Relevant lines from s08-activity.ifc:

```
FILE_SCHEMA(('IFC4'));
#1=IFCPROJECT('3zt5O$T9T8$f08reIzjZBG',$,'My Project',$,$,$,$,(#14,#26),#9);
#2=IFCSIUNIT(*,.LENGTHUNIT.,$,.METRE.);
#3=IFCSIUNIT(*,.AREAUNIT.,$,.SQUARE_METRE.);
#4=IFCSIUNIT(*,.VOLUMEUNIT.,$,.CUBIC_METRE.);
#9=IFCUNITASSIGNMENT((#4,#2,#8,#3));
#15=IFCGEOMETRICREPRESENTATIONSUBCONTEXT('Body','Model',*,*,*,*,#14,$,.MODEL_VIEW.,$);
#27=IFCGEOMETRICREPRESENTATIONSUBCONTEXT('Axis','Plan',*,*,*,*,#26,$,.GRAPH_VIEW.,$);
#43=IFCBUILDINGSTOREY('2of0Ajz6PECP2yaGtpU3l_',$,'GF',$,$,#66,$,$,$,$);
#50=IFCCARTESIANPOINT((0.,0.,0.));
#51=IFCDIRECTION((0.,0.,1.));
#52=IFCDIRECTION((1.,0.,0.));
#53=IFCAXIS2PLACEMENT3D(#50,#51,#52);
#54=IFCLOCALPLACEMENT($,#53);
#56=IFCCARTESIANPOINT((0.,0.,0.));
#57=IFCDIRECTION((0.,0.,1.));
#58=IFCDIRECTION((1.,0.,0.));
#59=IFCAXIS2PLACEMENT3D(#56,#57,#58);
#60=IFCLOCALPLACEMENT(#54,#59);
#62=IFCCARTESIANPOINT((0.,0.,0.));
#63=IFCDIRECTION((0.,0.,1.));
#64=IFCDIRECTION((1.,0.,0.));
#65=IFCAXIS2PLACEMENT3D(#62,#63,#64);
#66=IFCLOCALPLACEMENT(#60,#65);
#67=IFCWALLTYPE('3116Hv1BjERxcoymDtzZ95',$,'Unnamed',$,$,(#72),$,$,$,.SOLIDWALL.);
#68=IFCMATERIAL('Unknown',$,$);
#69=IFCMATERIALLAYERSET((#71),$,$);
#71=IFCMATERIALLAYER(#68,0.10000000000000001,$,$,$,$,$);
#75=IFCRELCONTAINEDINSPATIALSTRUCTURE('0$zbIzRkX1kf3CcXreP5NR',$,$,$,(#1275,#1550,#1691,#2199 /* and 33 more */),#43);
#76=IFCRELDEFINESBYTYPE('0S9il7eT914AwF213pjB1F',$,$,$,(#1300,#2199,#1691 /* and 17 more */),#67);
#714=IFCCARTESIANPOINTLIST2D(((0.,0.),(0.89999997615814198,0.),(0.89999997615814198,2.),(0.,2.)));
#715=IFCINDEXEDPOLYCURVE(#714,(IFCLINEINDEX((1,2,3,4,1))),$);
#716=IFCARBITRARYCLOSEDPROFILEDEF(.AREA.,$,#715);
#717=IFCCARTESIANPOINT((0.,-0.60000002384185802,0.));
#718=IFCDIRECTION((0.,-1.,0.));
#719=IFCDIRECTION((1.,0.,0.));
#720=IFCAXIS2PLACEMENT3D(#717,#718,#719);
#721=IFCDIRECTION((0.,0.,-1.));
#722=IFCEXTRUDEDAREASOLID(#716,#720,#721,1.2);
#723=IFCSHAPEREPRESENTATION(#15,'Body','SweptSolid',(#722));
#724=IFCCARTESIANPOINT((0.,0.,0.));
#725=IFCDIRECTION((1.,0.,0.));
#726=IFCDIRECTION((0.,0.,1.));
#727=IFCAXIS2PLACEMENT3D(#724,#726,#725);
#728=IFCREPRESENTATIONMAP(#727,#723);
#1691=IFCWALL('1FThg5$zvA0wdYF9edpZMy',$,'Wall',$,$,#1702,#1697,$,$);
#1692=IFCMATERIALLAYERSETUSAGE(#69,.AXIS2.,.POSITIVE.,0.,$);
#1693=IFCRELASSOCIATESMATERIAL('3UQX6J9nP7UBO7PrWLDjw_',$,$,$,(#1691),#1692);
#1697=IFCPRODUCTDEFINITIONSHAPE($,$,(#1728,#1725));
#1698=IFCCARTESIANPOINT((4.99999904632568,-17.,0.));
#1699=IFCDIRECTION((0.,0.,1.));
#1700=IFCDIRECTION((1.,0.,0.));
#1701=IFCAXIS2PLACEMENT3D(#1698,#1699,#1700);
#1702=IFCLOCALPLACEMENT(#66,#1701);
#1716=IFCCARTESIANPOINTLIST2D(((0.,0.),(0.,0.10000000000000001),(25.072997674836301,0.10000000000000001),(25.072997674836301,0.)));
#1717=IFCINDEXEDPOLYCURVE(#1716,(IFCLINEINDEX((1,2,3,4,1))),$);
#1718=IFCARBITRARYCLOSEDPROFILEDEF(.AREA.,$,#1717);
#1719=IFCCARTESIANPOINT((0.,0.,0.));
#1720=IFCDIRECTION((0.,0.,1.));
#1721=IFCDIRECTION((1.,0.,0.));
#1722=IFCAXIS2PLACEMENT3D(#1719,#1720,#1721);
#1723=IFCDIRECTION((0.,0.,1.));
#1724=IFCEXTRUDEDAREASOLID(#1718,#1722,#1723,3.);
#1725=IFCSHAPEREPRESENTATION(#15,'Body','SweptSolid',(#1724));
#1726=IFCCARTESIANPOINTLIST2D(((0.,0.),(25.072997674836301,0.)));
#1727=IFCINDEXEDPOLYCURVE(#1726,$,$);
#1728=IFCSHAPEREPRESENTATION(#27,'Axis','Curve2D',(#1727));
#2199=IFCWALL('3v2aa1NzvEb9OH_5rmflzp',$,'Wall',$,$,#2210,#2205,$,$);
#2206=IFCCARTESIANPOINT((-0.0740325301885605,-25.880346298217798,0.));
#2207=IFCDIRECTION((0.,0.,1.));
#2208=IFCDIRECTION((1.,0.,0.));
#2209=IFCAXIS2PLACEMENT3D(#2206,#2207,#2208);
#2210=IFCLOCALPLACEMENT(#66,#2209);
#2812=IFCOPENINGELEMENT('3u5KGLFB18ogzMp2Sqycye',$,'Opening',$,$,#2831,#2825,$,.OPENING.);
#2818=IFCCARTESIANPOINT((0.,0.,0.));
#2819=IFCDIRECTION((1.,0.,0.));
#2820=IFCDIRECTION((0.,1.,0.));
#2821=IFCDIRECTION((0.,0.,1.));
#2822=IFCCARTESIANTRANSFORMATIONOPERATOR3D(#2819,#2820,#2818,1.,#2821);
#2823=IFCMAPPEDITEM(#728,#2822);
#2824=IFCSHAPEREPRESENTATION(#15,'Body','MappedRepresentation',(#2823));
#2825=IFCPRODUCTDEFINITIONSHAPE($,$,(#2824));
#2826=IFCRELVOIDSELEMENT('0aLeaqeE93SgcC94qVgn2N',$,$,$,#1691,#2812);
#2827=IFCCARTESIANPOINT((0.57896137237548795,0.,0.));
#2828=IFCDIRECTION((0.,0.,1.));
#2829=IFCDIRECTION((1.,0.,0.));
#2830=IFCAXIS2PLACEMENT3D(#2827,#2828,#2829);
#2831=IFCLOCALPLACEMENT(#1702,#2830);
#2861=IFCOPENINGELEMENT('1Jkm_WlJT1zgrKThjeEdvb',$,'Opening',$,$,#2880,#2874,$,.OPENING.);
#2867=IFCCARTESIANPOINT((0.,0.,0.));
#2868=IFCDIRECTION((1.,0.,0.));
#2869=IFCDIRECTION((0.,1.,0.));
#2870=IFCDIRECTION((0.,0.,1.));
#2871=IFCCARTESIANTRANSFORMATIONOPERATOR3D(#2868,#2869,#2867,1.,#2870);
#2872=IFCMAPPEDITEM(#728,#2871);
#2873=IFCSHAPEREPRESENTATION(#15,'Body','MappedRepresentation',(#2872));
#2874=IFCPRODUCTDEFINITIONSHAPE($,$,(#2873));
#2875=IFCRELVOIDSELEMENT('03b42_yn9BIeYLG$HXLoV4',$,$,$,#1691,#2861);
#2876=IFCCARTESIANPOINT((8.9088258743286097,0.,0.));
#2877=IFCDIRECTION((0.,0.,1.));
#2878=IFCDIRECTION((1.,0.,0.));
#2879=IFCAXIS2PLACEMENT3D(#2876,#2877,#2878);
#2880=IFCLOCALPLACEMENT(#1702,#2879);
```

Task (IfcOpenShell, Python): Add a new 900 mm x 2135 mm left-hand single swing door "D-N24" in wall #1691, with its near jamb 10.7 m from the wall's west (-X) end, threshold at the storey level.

```python
import numpy as np
import ifcopenshell
import ifcopenshell.api.feature
import ifcopenshell.api.geometry
import ifcopenshell.api.root
import ifcopenshell.api.spatial
import ifcopenshell.geom
import ifcopenshell.util.element
import ifcopenshell.util.placement
import ifcopenshell.util.representation
import ifcopenshell.util.shape
import ifcopenshell.util.unit

model = ifcopenshell.open("s08-activity.ifc")
unit_scale = ifcopenshell.util.unit.calculate_unit_scale(model)
settings = ifcopenshell.geom.settings()


def volume(element):
    """Net volume in cubic metres, openings subtracted."""
    shape = ifcopenshell.geom.create_shape(settings, element)
    return ifcopenshell.util.shape.get_volume(shape.geometry)


wall = model.by_guid("1FThg5$zvA0wdYF9edpZMy")
storey = ifcopenshell.util.element.get_container(wall, ifc_class="IfcBuildingStorey")
context = ifcopenshell.util.representation.get_context(model, "Model", "Body", "MODEL_VIEW")
before = volume(wall)

width, height, from_end, sill = 0.9, 2.135, 10.7, 0.0  # metres

# The wall runs along its own X axis, and the end named is its -X end.
wall_shape = ifcopenshell.geom.create_shape(settings, wall)
x, y, z = ifcopenshell.util.shape.get_vertices(wall_shape.geometry).T
start = x.min() + from_end
face, thickness = float(y.min()), float(y.max() - y.min())
wall_matrix = ifcopenshell.util.placement.get_local_placement(wall.ObjectPlacement)
level = ifcopenshell.util.placement.get_local_placement(storey.ObjectPlacement)[2, 3]


def in_wall(x, y):
    """Placement at x, y metres in the wall's axes, at sill height."""
    matrix = wall_matrix.copy()
    matrix[:, 3] = wall_matrix @ np.array([x / unit_scale, y / unit_scale, 0.0, 1.0])
    matrix[2, 3] = level + sill / unit_scale
    return matrix


# Opening: a box that overshoots both wall faces by 50 mm.
opening = ifcopenshell.api.root.create_entity(model, ifc_class="IfcOpeningElement", predefined_type="OPENING")
box = ifcopenshell.api.geometry.add_wall_representation(
    model, context=context, length=width, height=height, thickness=thickness + 0.1
)
ifcopenshell.api.geometry.assign_representation(model, product=opening, representation=box)
ifcopenshell.api.geometry.edit_object_placement(model, product=opening, matrix=in_wall(start, face - 0.05), is_si=False)
ifcopenshell.api.feature.add_feature(model, feature=opening, element=wall)

door = ifcopenshell.api.root.create_entity(model, ifc_class="IfcDoor", name="D-N24", predefined_type="DOOR")
door.OverallWidth, door.OverallHeight = width / unit_scale, height / unit_scale
door.OperationType = "SINGLE_SWING_LEFT"
body = ifcopenshell.api.geometry.add_door_representation(
    model,
    context=context,
    overall_width=door.OverallWidth,
    overall_height=door.OverallHeight,
    operation_type="SINGLE_SWING_LEFT",
    lining_properties={"LiningDepth": thickness / unit_scale, "ThresholdDepth": thickness / unit_scale},
)
ifcopenshell.api.geometry.assign_representation(model, product=door, representation=body)
ifcopenshell.api.spatial.assign_container(model, products=[door], relating_structure=storey)
ifcopenshell.api.feature.add_filling(model, opening=opening, element=door)

# The lining spans the wall, so the door starts at the wall face.
ifcopenshell.api.geometry.edit_object_placement(model, product=door, matrix=in_wall(start, face), is_si=False)

after = volume(wall)

print(f"wall volume {before:.3f} -> {after:.3f} m3")

model.write("s08-activity-out.ifc")
```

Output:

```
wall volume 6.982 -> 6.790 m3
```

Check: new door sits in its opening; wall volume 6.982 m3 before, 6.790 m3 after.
